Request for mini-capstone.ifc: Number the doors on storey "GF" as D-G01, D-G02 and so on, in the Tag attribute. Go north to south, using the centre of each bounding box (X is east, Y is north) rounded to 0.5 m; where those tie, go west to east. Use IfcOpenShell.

First a look at what the model holds.

```python
import ifcopenshell
import ifcopenshell.util.element
import ifcopenshell.util.placement

model = ifcopenshell.open("mini-capstone.ifc")
print(model.schema)
storey = next(s for s in model.by_type("IfcBuildingStorey") if s.Name == "GF")
doors = [e for e in ifcopenshell.util.element.get_decomposition(storey) if e.is_a("IfcDoor")]
for e in sorted(doors, key=lambda e: e.id()):
    origin = ifcopenshell.util.placement.get_local_placement(e.ObjectPlacement)[:3, 3]
    print(e.id(), e.Tag, e.Name, origin.round(2) + 0.0, sep=" | ")
```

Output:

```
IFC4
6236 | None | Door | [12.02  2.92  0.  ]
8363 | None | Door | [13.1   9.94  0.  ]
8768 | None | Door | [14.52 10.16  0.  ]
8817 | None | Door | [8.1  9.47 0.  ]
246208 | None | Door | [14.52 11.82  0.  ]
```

```python
import ifcopenshell
import ifcopenshell.geom
import ifcopenshell.util.element
import ifcopenshell.util.shape

model = ifcopenshell.open("mini-capstone.ifc")
settings = ifcopenshell.geom.settings()
settings.set("use-world-coords", True)


def centre(element):
    shape = ifcopenshell.geom.create_shape(settings, element)
    return ifcopenshell.util.shape.get_bbox_centroid(shape.geometry)


storey = next(s for s in model.by_type("IfcBuildingStorey") if s.Name == "GF")
doors = [e for e in ifcopenshell.util.element.get_decomposition(storey) if e.is_a("IfcDoor")]

# Insertion points can sit at a corner or the storey origin, so sort by the geometry (in metres).
centres = {e: centre(e) for e in doors}
doors.sort(key=lambda e: (-round(centres[e][1] / 0.5), centres[e][0]))

for i, e in enumerate(doors, start=1):
    number = f"D-G{i:02d}"
    e.Tag = number
    print(e.id(), number)

model.write("mini-capstone_rev.ifc")
```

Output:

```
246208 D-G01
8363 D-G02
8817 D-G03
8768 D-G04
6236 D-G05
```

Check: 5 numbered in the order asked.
